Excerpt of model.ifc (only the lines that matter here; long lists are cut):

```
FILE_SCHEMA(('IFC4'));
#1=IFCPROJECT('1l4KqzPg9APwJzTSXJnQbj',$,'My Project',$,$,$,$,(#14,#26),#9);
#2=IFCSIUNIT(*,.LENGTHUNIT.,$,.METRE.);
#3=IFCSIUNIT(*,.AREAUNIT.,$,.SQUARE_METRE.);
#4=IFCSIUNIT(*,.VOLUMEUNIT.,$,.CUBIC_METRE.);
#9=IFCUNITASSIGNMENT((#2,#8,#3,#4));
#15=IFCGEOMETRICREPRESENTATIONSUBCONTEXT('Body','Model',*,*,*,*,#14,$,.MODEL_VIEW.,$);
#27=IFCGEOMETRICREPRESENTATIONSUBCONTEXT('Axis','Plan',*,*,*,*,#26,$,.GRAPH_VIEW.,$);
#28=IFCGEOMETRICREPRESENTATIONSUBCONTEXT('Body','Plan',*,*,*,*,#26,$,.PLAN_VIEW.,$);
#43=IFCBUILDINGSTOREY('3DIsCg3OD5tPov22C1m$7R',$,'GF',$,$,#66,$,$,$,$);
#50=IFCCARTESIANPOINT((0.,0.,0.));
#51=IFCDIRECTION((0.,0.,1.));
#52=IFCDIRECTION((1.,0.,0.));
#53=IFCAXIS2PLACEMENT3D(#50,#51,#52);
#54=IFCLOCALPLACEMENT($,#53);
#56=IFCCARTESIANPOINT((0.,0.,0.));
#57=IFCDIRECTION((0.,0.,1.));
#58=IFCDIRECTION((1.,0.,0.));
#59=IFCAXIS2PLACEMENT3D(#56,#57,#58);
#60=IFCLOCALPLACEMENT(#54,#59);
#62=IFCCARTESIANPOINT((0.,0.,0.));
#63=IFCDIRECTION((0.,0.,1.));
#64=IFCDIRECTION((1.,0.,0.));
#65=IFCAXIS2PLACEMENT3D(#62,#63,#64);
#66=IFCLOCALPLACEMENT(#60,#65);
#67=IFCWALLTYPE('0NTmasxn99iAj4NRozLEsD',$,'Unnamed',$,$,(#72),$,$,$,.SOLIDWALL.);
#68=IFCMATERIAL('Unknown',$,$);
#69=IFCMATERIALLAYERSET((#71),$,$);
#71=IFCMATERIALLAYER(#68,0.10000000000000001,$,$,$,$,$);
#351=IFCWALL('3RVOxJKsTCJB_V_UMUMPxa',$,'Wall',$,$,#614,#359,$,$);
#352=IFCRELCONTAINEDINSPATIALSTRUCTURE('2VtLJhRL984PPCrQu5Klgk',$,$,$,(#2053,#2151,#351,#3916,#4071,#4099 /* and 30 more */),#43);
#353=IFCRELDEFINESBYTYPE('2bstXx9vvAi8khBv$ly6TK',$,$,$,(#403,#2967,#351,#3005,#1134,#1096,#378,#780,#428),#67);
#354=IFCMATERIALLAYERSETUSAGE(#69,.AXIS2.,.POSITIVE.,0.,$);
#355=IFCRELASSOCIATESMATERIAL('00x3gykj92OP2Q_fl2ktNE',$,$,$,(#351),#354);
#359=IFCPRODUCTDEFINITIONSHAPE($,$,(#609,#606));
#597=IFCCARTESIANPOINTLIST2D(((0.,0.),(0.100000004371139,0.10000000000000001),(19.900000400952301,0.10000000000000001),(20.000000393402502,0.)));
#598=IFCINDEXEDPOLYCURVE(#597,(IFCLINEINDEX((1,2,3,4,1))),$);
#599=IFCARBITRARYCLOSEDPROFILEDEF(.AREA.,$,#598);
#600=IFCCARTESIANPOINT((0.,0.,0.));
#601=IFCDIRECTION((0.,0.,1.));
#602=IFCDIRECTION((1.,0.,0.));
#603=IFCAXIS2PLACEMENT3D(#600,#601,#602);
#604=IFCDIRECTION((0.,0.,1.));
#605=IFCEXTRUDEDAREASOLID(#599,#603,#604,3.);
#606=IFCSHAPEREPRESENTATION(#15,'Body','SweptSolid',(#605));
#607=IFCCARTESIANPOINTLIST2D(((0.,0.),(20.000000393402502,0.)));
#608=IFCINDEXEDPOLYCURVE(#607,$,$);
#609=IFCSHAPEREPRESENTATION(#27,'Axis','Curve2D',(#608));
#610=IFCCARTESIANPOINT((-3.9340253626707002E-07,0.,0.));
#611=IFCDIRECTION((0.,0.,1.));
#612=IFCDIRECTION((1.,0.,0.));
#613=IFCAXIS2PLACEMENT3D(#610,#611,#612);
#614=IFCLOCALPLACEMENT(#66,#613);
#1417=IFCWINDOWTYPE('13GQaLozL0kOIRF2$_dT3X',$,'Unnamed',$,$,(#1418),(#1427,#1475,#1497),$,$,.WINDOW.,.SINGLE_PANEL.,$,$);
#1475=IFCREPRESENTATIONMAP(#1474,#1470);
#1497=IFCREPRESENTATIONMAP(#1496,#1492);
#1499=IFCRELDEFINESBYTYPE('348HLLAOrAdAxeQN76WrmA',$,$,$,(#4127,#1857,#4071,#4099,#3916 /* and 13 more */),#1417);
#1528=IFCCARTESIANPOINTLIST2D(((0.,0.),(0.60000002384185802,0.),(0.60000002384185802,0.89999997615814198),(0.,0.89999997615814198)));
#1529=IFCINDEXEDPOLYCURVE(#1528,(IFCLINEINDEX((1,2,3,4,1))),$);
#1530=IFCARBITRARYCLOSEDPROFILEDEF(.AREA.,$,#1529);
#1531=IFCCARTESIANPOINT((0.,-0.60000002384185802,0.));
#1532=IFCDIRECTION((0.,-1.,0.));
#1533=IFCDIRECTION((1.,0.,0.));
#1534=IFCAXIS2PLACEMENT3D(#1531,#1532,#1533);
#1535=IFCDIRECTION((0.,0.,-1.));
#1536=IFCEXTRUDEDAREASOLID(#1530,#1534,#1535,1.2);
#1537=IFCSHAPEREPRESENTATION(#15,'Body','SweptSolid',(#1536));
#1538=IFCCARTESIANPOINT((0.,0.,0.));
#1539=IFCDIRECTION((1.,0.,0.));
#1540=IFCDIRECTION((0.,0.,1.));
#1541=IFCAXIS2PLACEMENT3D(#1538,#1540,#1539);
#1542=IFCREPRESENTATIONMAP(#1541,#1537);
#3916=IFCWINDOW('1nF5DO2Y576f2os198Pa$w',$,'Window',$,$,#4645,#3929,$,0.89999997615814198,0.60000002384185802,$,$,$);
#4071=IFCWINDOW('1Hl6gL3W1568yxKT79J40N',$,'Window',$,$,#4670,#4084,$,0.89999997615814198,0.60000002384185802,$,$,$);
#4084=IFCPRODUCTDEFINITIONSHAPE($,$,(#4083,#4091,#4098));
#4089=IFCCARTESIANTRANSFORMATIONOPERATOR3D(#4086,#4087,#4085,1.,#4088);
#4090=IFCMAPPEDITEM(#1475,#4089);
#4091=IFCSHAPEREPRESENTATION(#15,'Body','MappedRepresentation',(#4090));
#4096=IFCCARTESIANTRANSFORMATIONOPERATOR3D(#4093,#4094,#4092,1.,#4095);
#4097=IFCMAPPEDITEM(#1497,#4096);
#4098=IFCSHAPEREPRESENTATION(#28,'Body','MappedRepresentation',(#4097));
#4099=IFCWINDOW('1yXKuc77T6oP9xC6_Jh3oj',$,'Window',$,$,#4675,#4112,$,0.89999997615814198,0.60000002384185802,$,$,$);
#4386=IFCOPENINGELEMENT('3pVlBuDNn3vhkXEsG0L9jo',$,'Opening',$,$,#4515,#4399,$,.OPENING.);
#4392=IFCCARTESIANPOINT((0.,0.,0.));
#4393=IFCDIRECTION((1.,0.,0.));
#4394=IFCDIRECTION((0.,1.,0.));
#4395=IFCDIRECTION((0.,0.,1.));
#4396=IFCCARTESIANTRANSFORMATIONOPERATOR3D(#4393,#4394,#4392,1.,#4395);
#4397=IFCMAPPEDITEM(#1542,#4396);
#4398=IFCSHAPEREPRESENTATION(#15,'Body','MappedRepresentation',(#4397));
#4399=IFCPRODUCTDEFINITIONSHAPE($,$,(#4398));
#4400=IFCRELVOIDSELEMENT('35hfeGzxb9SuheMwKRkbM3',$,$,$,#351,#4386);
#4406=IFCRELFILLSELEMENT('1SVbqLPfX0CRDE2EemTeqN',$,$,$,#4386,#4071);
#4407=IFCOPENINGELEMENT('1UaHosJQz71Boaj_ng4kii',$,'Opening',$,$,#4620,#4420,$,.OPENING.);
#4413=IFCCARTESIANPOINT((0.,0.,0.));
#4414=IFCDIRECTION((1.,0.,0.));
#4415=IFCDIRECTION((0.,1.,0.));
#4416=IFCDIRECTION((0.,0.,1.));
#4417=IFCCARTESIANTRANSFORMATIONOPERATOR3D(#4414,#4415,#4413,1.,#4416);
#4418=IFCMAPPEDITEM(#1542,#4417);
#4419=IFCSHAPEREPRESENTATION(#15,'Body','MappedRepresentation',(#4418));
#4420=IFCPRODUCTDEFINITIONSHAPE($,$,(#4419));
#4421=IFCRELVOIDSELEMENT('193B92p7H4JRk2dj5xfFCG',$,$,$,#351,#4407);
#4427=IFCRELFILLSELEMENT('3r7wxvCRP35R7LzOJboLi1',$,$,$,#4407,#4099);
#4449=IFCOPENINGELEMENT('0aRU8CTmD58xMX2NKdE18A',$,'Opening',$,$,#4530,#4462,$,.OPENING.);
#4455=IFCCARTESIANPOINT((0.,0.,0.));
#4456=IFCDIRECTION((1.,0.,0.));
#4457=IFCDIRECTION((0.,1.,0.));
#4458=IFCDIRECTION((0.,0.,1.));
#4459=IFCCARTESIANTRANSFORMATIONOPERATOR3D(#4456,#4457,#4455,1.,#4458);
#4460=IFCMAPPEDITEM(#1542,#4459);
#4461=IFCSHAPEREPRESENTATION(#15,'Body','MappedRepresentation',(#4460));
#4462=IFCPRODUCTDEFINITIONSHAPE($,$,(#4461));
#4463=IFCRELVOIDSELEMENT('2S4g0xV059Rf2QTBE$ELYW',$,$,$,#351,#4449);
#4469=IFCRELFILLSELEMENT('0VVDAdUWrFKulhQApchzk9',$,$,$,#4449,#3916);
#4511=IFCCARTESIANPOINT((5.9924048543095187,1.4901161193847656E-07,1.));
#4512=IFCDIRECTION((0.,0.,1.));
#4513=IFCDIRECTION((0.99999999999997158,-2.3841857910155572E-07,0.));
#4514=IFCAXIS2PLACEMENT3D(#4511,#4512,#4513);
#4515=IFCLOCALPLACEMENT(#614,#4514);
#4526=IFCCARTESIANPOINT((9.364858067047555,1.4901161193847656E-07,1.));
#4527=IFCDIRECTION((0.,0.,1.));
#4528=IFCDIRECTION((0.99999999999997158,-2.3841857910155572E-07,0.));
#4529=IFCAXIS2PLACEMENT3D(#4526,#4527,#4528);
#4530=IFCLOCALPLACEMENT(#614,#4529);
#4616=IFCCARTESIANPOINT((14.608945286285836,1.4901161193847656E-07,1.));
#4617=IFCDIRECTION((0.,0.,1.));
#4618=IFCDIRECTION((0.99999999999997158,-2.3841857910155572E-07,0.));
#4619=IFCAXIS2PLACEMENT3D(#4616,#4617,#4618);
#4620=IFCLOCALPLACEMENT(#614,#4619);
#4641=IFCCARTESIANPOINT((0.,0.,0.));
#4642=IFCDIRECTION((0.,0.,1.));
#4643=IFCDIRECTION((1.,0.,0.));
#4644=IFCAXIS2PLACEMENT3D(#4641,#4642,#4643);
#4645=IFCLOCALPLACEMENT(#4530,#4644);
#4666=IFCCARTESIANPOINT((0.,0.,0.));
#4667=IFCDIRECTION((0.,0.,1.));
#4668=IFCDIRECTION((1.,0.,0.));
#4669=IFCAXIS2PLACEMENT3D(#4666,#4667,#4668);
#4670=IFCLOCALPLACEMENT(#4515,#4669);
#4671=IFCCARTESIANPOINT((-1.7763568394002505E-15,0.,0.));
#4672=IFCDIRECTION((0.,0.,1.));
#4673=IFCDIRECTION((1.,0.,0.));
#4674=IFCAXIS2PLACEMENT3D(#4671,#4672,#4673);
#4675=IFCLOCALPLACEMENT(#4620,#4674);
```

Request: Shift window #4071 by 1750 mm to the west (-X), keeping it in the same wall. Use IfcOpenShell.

```python
import ifcopenshell
import ifcopenshell.api.geometry
import ifcopenshell.util.placement

model = ifcopenshell.open("model.ifc")

window = model.by_guid("1Hl6gL3W1568yxKT79J40N")
opening = window.FillsVoids[0].RelatingOpeningElement
wall = opening.VoidsElements[0].RelatingBuildingElement

wall_matrix = ifcopenshell.util.placement.get_local_placement(wall.ObjectPlacement)
shift = wall_matrix[:3, 0] * -1.75
before = ifcopenshell.util.placement.get_local_placement(window.ObjectPlacement)[:3, 3].copy()

# The window is placed relative to its opening, so it follows when the opening moves.
matrix = ifcopenshell.util.placement.get_local_placement(opening.ObjectPlacement)
matrix[:3, 3] += shift
ifcopenshell.api.geometry.edit_object_placement(
    model, product=opening, matrix=matrix, is_si=False, should_transform_children=True
)

after = ifcopenshell.util.placement.get_local_placement(window.ObjectPlacement)[:3, 3]
print("window moved by", (after - before).round(3) + 0.0)

model.write("model_edited.ifc")
```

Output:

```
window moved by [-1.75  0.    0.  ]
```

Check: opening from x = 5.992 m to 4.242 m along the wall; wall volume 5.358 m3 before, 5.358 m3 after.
